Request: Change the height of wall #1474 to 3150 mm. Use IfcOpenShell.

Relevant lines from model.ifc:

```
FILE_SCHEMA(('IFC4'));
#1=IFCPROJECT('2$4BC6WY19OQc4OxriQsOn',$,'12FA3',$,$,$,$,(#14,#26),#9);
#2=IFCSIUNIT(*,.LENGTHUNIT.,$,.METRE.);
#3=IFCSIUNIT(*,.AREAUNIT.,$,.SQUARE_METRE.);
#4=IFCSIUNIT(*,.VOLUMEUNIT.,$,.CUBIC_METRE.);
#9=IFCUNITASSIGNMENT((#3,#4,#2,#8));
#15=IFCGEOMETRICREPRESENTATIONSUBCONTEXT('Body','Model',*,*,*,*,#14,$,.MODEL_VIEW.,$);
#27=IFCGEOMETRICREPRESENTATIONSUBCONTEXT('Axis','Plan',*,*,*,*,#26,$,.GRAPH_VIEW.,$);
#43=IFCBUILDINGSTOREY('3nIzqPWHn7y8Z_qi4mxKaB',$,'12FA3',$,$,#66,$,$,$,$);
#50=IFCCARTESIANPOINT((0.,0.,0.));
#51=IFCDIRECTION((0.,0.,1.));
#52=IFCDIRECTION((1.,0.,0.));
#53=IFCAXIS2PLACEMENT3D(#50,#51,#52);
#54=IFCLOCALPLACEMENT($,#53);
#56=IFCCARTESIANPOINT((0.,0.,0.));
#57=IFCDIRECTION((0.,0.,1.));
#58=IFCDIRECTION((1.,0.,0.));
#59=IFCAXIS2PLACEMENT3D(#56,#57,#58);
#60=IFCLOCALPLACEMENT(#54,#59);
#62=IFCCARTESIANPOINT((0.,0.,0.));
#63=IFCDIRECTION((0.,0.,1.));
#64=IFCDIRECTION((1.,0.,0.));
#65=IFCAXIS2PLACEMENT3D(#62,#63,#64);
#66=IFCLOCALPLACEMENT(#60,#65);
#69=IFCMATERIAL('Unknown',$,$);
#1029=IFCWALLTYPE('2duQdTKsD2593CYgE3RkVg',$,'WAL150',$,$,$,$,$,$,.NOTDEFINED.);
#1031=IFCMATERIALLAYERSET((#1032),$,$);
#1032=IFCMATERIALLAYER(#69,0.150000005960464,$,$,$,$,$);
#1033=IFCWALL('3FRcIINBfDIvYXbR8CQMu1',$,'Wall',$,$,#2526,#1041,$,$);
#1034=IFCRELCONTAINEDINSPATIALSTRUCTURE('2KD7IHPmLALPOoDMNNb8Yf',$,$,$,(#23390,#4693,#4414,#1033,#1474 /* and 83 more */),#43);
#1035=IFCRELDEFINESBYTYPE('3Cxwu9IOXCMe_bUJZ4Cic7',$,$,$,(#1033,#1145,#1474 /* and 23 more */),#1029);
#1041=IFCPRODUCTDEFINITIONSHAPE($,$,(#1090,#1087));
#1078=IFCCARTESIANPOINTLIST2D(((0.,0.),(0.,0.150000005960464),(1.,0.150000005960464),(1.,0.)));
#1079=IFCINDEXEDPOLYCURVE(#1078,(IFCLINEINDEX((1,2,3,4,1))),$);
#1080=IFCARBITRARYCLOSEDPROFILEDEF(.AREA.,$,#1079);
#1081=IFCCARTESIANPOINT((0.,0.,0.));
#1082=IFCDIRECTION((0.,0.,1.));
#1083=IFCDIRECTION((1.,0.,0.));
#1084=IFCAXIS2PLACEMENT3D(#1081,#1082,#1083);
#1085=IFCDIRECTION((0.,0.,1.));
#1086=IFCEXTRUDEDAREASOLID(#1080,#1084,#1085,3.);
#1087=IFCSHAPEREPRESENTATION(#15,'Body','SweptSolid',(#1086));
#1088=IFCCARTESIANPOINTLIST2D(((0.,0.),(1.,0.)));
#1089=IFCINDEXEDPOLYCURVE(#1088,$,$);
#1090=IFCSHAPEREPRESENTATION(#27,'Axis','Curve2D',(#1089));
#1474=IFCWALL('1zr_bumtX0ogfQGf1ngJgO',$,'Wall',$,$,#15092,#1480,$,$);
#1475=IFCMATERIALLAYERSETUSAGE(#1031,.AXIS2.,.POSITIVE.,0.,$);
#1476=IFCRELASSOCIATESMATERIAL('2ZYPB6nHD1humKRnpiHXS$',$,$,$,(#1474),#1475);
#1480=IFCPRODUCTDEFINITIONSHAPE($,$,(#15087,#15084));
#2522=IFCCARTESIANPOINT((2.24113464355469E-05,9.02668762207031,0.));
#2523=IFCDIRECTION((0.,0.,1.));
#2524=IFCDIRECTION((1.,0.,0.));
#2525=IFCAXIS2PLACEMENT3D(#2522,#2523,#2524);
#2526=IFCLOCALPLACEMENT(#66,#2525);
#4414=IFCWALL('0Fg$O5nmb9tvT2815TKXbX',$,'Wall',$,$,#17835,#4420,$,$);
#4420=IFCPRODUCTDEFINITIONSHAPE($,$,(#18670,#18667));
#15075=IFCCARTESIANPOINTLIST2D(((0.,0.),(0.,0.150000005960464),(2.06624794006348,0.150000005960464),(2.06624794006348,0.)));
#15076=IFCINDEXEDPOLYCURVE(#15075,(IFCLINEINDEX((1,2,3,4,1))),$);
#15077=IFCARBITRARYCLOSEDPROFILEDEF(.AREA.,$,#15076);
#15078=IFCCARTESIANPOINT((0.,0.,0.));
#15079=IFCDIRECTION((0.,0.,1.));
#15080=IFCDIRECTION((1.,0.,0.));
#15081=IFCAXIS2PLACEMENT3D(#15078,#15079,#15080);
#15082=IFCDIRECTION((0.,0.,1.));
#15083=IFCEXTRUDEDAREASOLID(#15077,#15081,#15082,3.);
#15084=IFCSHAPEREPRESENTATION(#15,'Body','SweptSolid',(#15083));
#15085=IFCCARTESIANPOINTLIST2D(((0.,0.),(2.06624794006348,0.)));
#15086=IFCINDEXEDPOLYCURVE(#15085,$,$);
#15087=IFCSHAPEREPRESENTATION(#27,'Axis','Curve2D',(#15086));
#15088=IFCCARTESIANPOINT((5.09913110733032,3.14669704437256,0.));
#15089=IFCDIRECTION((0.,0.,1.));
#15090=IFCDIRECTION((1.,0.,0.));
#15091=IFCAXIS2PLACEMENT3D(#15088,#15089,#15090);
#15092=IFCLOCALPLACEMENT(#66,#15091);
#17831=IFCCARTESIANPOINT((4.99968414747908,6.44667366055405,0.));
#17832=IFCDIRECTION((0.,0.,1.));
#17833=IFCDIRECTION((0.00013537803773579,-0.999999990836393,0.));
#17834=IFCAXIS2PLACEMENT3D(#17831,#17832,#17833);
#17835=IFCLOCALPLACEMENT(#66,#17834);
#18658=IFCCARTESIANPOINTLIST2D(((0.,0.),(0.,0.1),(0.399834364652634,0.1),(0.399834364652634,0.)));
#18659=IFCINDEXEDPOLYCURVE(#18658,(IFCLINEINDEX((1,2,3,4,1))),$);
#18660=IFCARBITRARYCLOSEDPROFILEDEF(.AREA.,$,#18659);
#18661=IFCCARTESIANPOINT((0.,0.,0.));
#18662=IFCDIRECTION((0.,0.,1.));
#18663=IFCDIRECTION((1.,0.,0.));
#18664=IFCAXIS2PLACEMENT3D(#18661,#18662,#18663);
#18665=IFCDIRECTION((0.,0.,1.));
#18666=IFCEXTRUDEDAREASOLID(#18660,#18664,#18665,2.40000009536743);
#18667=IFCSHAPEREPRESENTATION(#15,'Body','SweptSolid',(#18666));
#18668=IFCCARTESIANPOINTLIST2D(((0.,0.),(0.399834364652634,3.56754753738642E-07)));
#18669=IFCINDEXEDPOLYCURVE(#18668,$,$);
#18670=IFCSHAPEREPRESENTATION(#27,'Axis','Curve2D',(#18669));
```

```python
import ifcopenshell
import ifcopenshell.geom
import ifcopenshell.util.representation
import ifcopenshell.util.shape

model = ifcopenshell.open("model.ifc")
settings = ifcopenshell.geom.settings()


def volume(element):
    """Net volume in cubic metres, openings subtracted."""
    shape = ifcopenshell.geom.create_shape(settings, element)
    return ifcopenshell.util.shape.get_volume(shape.geometry)


wall = model.by_guid("1zr_bumtX0ogfQGf1ngJgO")
before = volume(wall)

body = ifcopenshell.util.representation.get_representation(wall, "Model", "Body")
solid = body.Items[0]
old_height = solid.Depth
solid.Depth = 3.15
after = volume(wall)

print(f"height {old_height:g} -> {solid.Depth:g}, volume {before:.3f} -> {after:.3f} m3")

model.write("model_v2.ifc")
```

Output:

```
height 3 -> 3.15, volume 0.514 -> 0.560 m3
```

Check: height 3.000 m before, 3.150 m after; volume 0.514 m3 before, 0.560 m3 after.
